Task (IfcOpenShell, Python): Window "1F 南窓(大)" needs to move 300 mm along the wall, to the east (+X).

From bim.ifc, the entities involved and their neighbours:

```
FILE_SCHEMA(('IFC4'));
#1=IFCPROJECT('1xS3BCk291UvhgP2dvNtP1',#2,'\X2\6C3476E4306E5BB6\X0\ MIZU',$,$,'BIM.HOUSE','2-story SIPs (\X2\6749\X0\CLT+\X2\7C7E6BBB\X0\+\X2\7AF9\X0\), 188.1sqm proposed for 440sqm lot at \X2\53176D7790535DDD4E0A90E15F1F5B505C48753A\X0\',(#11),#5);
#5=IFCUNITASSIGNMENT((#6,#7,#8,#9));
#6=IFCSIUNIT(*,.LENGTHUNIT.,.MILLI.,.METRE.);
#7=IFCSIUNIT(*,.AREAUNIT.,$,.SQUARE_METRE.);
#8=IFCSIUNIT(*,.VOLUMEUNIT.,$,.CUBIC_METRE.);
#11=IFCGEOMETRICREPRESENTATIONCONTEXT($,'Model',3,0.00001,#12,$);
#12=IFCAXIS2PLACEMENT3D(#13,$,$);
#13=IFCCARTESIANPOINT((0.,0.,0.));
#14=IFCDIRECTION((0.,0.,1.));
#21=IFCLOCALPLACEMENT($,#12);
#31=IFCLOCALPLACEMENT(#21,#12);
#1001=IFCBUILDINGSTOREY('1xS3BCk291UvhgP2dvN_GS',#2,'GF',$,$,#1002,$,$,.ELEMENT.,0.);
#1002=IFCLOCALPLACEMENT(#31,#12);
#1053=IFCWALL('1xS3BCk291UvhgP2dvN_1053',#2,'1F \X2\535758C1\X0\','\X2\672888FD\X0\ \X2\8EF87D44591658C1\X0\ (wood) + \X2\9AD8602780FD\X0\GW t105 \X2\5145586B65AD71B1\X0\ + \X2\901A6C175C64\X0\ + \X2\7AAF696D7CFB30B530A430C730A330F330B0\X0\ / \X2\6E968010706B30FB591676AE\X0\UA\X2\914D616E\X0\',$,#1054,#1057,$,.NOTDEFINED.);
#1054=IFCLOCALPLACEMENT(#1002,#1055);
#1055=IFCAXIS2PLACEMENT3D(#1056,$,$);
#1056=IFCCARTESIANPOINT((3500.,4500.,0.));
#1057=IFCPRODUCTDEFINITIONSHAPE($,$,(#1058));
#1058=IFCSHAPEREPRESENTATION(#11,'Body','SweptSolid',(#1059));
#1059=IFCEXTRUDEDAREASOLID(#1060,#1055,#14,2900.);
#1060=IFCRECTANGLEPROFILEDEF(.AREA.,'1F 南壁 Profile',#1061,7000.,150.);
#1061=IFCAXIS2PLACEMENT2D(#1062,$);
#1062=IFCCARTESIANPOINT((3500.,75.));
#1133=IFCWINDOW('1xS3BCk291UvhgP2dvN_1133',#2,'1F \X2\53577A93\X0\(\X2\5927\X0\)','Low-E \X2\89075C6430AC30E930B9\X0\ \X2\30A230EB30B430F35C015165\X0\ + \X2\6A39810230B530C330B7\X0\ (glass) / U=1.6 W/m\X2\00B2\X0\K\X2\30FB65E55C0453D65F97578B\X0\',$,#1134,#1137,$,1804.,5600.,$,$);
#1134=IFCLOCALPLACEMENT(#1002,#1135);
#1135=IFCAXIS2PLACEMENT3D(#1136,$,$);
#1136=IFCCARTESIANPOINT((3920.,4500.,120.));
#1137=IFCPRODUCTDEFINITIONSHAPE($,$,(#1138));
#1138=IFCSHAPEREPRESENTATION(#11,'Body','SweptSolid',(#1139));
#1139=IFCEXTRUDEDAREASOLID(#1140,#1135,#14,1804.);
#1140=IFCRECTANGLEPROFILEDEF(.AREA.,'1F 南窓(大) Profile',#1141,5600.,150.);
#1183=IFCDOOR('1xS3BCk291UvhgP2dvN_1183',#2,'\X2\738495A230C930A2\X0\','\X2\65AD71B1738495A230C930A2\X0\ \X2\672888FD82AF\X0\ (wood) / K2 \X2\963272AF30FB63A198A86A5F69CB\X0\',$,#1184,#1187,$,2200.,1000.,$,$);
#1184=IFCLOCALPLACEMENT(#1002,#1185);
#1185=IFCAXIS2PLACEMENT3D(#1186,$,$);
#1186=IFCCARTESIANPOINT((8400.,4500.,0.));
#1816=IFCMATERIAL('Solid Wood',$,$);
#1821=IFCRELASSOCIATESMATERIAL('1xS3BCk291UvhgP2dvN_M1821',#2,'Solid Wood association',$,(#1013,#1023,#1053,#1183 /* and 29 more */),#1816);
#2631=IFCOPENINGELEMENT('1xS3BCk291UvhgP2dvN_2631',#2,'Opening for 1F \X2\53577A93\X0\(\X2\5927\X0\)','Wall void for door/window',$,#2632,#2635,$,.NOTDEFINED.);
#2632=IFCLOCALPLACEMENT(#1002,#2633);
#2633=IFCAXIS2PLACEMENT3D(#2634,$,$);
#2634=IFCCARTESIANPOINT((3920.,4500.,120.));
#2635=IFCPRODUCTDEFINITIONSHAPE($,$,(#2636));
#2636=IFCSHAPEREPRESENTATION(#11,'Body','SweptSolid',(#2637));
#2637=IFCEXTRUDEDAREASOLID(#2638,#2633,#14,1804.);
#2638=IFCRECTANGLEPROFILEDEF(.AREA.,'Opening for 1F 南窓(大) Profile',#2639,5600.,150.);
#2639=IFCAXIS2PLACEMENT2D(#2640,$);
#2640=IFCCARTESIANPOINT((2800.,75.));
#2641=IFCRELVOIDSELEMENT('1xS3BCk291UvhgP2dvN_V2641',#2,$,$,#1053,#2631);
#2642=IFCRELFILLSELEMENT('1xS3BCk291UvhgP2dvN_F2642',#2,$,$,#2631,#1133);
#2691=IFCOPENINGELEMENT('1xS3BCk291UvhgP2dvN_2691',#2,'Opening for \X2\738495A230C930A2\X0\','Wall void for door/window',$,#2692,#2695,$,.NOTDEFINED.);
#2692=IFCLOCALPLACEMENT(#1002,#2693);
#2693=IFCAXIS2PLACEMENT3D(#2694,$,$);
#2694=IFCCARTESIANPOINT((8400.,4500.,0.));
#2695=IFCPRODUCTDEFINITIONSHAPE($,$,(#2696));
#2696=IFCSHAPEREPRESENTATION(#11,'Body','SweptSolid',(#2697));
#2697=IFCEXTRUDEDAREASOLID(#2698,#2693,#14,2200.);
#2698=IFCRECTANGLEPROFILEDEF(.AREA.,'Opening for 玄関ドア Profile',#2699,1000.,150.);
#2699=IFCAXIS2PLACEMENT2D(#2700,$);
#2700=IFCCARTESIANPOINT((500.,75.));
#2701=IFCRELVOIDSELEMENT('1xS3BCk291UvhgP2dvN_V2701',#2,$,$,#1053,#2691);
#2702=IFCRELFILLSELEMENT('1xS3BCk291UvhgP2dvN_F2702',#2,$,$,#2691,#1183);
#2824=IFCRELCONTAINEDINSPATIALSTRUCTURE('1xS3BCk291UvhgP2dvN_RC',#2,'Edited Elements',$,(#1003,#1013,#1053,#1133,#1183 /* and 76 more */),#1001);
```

```python
import ifcopenshell
import ifcopenshell.api.geometry
import ifcopenshell.util.placement

model = ifcopenshell.open("bim.ifc")

window = model.by_guid("1xS3BCk291UvhgP2dvN_1133")
opening = window.FillsVoids[0].RelatingOpeningElement
wall = opening.VoidsElements[0].RelatingBuildingElement

wall_matrix = ifcopenshell.util.placement.get_local_placement(wall.ObjectPlacement)
shift = wall_matrix[:3, 0] * 300.0
before = ifcopenshell.util.placement.get_local_placement(window.ObjectPlacement)[:3, 3].copy()

# The window is not placed relative to its opening, so move both.
for product in (opening, window):
    matrix = ifcopenshell.util.placement.get_local_placement(product.ObjectPlacement)
    matrix[:3, 3] += shift
    ifcopenshell.api.geometry.edit_object_placement(model, product=product, matrix=matrix, is_si=False)

after = ifcopenshell.util.placement.get_local_placement(window.ObjectPlacement)[:3, 3]
print("window moved by", (after - before).round(3) + 0.0)

model.write("bim_updated.ifc")
```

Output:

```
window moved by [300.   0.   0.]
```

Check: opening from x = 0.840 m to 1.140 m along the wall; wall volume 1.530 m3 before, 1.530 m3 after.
